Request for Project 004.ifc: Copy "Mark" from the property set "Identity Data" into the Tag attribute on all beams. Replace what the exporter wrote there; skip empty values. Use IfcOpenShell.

First a look at what the model holds.

```python
import ifcopenshell
import ifcopenshell.util.element

model = ifcopenshell.open("Project 004.ifc")
print(model.schema)
beams = model.by_type("IfcBeam")
print(len(beams), "beams")
for e in beams[:8]:
    source = ifcopenshell.util.element.get_pset(e, "Identity Data", "Mark")
    target = e.Tag
    print(e.id(), repr(source), repr(target), sep=" | ")
```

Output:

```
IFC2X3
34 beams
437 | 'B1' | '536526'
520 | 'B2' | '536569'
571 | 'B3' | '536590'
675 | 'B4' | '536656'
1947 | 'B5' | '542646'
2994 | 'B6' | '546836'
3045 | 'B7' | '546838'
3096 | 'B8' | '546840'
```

```python
import ifcopenshell
import ifcopenshell.util.element

model = ifcopenshell.open("Project 004.ifc")

count = 0
for e in model.by_type("IfcBeam"):
    value = ifcopenshell.util.element.get_pset(e, "Identity Data", "Mark")
    current = e.Tag
    if not value or not value.strip() or current == value:
        continue
    e.Tag = value
    count += 1

print(count, "beams updated")

model.write("Project 004_updated.ifc")
```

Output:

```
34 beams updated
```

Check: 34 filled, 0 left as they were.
